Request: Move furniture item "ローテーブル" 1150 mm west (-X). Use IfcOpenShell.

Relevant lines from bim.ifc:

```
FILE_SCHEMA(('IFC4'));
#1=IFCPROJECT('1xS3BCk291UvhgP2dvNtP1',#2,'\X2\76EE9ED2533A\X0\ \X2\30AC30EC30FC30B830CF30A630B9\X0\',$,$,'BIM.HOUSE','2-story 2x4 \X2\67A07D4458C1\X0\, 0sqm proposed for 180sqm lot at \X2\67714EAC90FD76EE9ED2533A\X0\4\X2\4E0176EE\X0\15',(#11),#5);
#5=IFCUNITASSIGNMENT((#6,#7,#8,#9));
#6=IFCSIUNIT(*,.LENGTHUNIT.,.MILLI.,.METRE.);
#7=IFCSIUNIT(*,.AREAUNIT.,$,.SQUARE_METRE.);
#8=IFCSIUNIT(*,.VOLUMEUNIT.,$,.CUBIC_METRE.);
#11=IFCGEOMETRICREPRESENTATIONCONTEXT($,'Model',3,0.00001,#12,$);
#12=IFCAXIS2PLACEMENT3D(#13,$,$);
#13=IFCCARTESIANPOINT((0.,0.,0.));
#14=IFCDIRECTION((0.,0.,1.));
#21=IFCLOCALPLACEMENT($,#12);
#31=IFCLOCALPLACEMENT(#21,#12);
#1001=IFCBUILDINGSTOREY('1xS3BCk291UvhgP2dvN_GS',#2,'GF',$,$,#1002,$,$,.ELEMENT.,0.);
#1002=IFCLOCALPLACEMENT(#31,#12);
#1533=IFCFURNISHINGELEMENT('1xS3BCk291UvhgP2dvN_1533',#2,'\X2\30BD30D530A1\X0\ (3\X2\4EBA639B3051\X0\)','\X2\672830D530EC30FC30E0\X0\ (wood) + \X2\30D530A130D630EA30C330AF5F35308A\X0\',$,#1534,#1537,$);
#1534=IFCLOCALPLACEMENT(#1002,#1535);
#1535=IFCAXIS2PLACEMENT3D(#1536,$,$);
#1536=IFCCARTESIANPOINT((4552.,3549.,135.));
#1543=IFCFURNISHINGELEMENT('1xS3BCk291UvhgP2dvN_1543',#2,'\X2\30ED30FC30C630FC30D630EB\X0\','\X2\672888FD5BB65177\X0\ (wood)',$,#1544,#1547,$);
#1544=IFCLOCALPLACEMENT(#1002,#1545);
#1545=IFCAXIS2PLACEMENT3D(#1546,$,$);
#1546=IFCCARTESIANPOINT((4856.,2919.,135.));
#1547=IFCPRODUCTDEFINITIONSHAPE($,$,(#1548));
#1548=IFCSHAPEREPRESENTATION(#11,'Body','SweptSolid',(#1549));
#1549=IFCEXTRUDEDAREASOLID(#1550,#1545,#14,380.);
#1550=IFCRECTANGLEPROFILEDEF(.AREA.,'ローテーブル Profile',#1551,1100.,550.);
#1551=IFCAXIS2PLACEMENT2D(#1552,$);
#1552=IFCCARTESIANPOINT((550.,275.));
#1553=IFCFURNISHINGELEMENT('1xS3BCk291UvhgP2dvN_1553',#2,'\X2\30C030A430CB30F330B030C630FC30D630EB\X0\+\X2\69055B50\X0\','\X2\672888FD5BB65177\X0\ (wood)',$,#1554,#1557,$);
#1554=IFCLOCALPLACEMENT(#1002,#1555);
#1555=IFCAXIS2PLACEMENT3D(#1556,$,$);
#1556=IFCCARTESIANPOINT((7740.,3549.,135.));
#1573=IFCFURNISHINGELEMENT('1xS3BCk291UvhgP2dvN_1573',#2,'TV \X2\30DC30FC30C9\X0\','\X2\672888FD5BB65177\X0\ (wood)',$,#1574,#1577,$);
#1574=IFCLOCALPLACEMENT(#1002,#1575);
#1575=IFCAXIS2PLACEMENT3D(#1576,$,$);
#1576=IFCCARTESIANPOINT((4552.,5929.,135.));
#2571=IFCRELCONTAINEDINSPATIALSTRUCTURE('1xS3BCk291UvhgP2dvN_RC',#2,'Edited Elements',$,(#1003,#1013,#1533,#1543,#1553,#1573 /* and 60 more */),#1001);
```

```python
import ifcopenshell
import ifcopenshell.api.geometry
import ifcopenshell.util.placement
import ifcopenshell.util.unit

model = ifcopenshell.open("bim.ifc")
unit_scale = ifcopenshell.util.unit.calculate_unit_scale(model)

item = model.by_id(1543)
matrix = ifcopenshell.util.placement.get_local_placement(item.ObjectPlacement)
matrix[0, 3] -= 1.15 / unit_scale
ifcopenshell.api.geometry.edit_object_placement(model, product=item, matrix=matrix, is_si=False)

print(ifcopenshell.util.placement.get_local_placement(item.ObjectPlacement).round(3) + 0.0)

model.write("bim_edited.ifc")
```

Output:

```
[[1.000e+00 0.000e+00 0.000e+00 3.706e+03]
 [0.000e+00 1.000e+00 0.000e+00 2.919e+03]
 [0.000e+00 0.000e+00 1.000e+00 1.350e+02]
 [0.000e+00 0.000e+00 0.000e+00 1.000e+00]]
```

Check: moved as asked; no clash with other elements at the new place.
